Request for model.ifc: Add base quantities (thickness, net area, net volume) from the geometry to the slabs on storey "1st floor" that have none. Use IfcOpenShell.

First a look at what the model holds.

```python
import ifcopenshell
import ifcopenshell.util.element
import ifcopenshell.util.unit

model = ifcopenshell.open("model.ifc")
print(model.schema)
for unit_type in ("LENGTHUNIT", "AREAUNIT", "VOLUMEUNIT"):
    print(unit_type, ifcopenshell.util.unit.calculate_unit_scale(model, unit_type))
storey = next(s for s in model.by_type("IfcBuildingStorey") if s.Name == "1st floor")
slabs = [e for e in ifcopenshell.util.element.get_decomposition(storey) if e.is_a("IfcSlab")]
for e in sorted(slabs, key=lambda e: e.id()):
    print(e.id(), e.is_a(), e.Name, list(ifcopenshell.util.element.get_psets(e, qtos_only=True)), sep=" | ")
```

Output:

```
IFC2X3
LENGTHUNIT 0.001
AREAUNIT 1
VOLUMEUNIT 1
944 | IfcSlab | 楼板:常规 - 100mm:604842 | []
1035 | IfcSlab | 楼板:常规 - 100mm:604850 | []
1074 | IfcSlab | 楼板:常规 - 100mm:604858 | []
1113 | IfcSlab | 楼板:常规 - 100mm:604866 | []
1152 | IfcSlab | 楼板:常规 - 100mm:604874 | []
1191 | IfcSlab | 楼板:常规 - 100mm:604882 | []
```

```python
import ifcopenshell
import ifcopenshell.api.pset
import ifcopenshell.geom
import ifcopenshell.util.element
import ifcopenshell.util.shape
import ifcopenshell.util.unit

model = ifcopenshell.open("model.ifc")
unit_scale = ifcopenshell.util.unit.calculate_unit_scale(model)
area_scale = ifcopenshell.util.unit.calculate_unit_scale(model, "AREAUNIT")
volume_scale = ifcopenshell.util.unit.calculate_unit_scale(model, "VOLUMEUNIT")
settings = ifcopenshell.geom.settings()

storey = next(s for s in model.by_type("IfcBuildingStorey") if s.Name == "1st floor")
slabs = [e for e in ifcopenshell.util.element.get_decomposition(storey) if e.is_a("IfcSlab")]

for e in sorted(slabs, key=lambda e: e.id()):
    if ifcopenshell.util.element.get_psets(e, qtos_only=True, should_inherit=False):
        continue
    # Geometry comes back in metres, in the element's own axes.
    shape = ifcopenshell.geom.create_shape(settings, e)
    values = {
        "Width": ifcopenshell.util.shape.get_z(shape.geometry) / unit_scale,
        "NetArea": ifcopenshell.util.shape.get_footprint_area(shape.geometry) / area_scale,
        "NetVolume": ifcopenshell.util.shape.get_volume(shape.geometry) / volume_scale,
    }
    qto = ifcopenshell.api.pset.add_qto(model, product=e, name="BaseQuantities")
    ifcopenshell.api.pset.edit_qto(model, qto=qto, properties=values)
    print(e.id(), {k: round(v, 3) for k, v in values.items()})

model.write("model_rev.ifc")
```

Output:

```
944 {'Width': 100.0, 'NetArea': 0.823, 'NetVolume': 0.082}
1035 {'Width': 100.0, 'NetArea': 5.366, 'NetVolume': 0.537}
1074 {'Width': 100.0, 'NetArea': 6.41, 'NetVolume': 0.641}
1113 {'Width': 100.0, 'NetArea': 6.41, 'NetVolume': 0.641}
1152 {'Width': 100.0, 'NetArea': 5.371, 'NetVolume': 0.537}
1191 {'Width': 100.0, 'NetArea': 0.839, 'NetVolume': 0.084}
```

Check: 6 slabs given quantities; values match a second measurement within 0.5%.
